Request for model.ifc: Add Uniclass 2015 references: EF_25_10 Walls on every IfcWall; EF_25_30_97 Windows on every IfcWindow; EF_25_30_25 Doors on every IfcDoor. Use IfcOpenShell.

First a look at what the model holds.

```python
import ifcopenshell

model = ifcopenshell.open("model.ifc")
print(model.schema)
print("classifications:", [c.Name for c in model.by_type("IfcClassification")])
for ifc_class in ("IfcDoor", "IfcRoof", "IfcStair", "IfcWall", "IfcWindow"):
    print(ifc_class, len(model.by_type(ifc_class)))
```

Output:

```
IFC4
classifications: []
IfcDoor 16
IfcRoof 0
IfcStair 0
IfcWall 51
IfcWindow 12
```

```python
import ifcopenshell
import ifcopenshell.api.classification

model = ifcopenshell.open("model.ifc")

system = ifcopenshell.api.classification.add_classification(model, classification="Uniclass 2015")

codes = {
    "IfcWall": ("EF_25_10", "Walls"),
    "IfcWindow": ("EF_25_30_97", "Windows"),
    "IfcDoor": ("EF_25_30_25", "Doors"),
}
for ifc_class, (code, name) in codes.items():
    products = model.by_type(ifc_class)
    ifcopenshell.api.classification.add_reference(
        model, products=products, classification=system, identification=code, name=name
    )
    print(code, len(products))

model.write("model_updated.ifc")
```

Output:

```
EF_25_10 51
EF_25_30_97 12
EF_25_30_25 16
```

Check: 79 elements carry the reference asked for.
